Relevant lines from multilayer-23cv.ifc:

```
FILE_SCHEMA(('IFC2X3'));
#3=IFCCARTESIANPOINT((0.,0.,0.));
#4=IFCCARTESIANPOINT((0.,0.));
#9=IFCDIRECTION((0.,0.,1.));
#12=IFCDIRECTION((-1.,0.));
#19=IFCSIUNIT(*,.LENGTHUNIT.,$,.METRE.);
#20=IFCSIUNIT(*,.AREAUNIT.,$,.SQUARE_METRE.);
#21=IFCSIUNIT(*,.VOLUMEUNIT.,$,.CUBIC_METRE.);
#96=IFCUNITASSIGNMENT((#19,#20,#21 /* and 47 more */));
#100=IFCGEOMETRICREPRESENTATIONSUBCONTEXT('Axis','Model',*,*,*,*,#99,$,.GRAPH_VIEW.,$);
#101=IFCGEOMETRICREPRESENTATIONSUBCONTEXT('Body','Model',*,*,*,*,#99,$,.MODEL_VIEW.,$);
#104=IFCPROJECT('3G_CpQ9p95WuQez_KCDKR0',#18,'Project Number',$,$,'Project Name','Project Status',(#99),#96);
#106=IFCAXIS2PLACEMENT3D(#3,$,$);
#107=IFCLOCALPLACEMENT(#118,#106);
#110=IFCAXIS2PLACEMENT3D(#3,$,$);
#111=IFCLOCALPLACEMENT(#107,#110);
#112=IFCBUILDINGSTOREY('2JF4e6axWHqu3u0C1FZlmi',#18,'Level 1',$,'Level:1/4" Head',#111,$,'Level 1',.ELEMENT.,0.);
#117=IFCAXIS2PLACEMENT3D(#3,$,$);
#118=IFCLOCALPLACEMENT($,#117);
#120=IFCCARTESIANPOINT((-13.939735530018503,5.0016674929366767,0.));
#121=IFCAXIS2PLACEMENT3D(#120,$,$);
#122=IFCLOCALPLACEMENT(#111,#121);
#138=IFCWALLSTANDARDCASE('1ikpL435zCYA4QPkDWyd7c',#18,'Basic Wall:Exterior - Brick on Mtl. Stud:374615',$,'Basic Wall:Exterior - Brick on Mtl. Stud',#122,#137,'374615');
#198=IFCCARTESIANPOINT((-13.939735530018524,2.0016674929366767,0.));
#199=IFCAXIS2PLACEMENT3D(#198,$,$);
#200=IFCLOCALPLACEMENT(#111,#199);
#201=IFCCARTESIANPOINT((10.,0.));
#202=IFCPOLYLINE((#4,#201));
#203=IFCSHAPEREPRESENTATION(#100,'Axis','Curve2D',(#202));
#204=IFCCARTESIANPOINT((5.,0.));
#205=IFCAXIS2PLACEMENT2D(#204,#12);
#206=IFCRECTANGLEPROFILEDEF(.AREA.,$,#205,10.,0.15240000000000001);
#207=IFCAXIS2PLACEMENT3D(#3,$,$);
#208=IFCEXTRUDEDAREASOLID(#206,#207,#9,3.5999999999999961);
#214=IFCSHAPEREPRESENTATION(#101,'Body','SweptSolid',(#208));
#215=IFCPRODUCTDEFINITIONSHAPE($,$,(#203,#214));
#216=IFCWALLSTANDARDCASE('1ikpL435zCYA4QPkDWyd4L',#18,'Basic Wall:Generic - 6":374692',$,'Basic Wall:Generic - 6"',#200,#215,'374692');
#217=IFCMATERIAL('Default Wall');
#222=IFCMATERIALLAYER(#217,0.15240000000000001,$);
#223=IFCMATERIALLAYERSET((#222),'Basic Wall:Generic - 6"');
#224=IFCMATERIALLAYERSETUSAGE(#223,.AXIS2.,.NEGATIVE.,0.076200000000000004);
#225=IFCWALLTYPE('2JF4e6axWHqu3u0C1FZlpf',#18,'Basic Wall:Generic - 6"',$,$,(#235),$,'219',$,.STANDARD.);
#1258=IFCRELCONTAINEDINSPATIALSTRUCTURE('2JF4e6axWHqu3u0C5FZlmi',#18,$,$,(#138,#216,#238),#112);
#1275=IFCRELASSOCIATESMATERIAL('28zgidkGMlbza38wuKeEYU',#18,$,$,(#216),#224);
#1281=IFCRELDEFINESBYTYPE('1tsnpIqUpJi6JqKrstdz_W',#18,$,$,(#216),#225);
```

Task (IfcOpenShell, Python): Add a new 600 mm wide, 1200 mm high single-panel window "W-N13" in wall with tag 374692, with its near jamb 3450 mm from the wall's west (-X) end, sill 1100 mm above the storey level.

```python
import numpy as np
import ifcopenshell
import ifcopenshell.api.feature
import ifcopenshell.api.geometry
import ifcopenshell.api.root
import ifcopenshell.api.spatial
import ifcopenshell.api.type
import ifcopenshell.geom
import ifcopenshell.util.element
import ifcopenshell.util.placement
import ifcopenshell.util.representation
import ifcopenshell.util.shape
import ifcopenshell.util.unit

model = ifcopenshell.open("multilayer-23cv.ifc")
unit_scale = ifcopenshell.util.unit.calculate_unit_scale(model)
settings = ifcopenshell.geom.settings()


def volume(element):
    """Net volume in cubic metres, openings subtracted."""
    shape = ifcopenshell.geom.create_shape(settings, element)
    return ifcopenshell.util.shape.get_volume(shape.geometry)


wall = model.by_guid("1ikpL435zCYA4QPkDWyd4L")
storey = ifcopenshell.util.element.get_container(wall, ifc_class="IfcBuildingStorey")
context = ifcopenshell.util.representation.get_context(model, "Model", "Body", "MODEL_VIEW")
before = volume(wall)

width, height, from_end, sill = 0.6, 1.2, 3.45, 1.1  # metres

# The wall runs along its own X axis, and the end named is its -X end.
wall_shape = ifcopenshell.geom.create_shape(settings, wall)
x, y, z = ifcopenshell.util.shape.get_vertices(wall_shape.geometry).T
start = x.min() + from_end
face, thickness = float(y.min()), float(y.max() - y.min())
wall_matrix = ifcopenshell.util.placement.get_local_placement(wall.ObjectPlacement)
level = ifcopenshell.util.placement.get_local_placement(storey.ObjectPlacement)[2, 3]


def in_wall(x, y):
    """Placement at x, y metres in the wall's axes, at sill height."""
    matrix = wall_matrix.copy()
    matrix[:, 3] = wall_matrix @ np.array([x / unit_scale, y / unit_scale, 0.0, 1.0])
    matrix[2, 3] = level + sill / unit_scale
    return matrix


# Opening: a box that overshoots both wall faces by 50 mm.
opening = ifcopenshell.api.root.create_entity(model, ifc_class="IfcOpeningElement")
box = ifcopenshell.api.geometry.add_wall_representation(
    model, context=context, length=width, height=height, thickness=thickness + 0.1
)
ifcopenshell.api.geometry.assign_representation(model, product=opening, representation=box)
ifcopenshell.api.geometry.edit_object_placement(model, product=opening, matrix=in_wall(start, face - 0.05), is_si=False)
ifcopenshell.api.feature.add_feature(model, feature=opening, element=wall)

window = ifcopenshell.api.root.create_entity(model, ifc_class="IfcWindow", name="W-N13")
window.OverallWidth, window.OverallHeight = width / unit_scale, height / unit_scale
body = ifcopenshell.api.geometry.add_window_representation(
    model,
    context=context,
    overall_width=window.OverallWidth,
    overall_height=window.OverallHeight,
    partition_type="SINGLE_PANEL",
)
ifcopenshell.api.geometry.assign_representation(model, product=window, representation=body)
ifcopenshell.api.spatial.assign_container(model, products=[window], relating_structure=storey)
fills = ifcopenshell.api.feature.add_filling(model, opening=opening, element=window)
fills.OwnerHistory = window.OwnerHistory  # required in IFC2X3

# IFC2X3 keeps the operation on the window style.
style = ifcopenshell.api.root.create_entity(model, ifc_class="IfcWindowStyle", name="W-N13")
style.OperationType, style.ConstructionType = "SINGLE_PANEL", "NOTDEFINED"
style.ParameterTakesPrecedence = style.Sizeable = False
ifcopenshell.api.type.assign_type(model, related_objects=[window], relating_type=style)

# Centre the window in the wall's thickness.
ifcopenshell.api.geometry.edit_object_placement(model, product=window, matrix=in_wall(start, face), is_si=False)
window_shape = ifcopenshell.geom.create_shape(settings, window)
depth = ifcopenshell.util.shape.get_vertices(window_shape.geometry)[:, 1]
offset = face + thickness / 2 - (depth.min() + depth.max()) / 2
ifcopenshell.api.geometry.edit_object_placement(model, product=window, matrix=in_wall(start, offset), is_si=False)

after = volume(wall)

print(f"wall volume {before:.3f} -> {after:.3f} m3")

model.write("multilayer-23cv_rev.ifc")
```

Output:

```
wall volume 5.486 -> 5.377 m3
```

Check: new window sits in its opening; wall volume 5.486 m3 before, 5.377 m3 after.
